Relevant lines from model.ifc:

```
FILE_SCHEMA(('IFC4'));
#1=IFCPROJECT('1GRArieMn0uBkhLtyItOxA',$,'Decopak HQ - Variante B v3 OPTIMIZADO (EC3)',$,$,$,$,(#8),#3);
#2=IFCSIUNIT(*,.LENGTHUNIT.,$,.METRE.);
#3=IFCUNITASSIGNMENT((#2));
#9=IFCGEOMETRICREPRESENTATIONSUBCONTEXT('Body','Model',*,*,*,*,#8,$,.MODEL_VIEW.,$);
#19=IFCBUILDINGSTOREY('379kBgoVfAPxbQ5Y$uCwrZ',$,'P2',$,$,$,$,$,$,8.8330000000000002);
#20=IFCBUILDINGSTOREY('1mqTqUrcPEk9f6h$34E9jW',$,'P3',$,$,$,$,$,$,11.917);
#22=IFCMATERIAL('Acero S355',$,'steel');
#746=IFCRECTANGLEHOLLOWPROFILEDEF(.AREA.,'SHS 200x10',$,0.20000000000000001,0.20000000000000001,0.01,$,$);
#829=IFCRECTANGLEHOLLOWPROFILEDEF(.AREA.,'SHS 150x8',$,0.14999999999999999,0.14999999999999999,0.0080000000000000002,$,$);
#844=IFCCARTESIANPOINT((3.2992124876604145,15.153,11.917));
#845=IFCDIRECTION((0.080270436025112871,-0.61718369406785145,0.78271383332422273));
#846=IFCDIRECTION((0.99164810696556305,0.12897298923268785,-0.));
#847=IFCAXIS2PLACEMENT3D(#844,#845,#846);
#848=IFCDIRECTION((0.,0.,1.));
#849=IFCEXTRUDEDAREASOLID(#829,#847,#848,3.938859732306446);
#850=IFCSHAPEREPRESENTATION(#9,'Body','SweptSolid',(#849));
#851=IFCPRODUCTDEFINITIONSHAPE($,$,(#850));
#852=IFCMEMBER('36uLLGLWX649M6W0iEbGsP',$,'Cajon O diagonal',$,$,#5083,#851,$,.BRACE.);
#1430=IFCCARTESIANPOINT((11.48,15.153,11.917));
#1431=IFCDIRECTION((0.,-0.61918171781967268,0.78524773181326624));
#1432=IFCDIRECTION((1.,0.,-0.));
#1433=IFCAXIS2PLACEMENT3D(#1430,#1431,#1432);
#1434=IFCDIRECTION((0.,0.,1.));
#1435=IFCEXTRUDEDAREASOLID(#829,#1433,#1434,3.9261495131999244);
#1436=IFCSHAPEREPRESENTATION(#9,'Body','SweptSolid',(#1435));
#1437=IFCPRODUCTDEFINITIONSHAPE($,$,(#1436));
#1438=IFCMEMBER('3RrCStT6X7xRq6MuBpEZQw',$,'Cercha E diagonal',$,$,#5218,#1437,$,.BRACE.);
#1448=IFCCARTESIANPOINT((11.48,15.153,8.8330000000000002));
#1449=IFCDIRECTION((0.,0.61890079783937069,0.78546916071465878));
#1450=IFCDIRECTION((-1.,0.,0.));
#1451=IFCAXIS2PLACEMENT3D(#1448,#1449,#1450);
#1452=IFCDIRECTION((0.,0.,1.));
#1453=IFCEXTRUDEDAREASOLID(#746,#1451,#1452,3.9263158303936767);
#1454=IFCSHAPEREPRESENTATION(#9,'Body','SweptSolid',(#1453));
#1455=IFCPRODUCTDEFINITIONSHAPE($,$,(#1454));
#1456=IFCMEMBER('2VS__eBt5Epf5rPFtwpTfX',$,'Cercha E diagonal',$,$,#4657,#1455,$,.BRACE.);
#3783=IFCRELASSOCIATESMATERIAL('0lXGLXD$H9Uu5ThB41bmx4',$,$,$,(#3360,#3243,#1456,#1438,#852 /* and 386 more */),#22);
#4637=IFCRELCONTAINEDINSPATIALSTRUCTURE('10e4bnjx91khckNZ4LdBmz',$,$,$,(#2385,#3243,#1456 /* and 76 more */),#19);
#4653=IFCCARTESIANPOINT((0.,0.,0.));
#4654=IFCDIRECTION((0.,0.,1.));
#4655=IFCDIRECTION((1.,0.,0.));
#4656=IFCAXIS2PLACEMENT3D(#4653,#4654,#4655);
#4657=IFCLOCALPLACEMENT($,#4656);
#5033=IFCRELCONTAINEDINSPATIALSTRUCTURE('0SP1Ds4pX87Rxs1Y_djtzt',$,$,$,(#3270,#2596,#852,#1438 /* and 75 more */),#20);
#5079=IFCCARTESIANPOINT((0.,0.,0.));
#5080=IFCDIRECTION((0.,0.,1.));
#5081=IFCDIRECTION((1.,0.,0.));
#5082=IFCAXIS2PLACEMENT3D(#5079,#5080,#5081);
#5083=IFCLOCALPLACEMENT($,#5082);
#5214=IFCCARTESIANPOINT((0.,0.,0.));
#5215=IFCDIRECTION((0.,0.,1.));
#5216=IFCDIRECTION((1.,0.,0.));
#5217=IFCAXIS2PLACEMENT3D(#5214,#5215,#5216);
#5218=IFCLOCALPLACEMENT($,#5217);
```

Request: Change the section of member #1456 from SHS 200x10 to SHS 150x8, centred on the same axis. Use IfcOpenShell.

```python
import ifcopenshell
import ifcopenshell.util.element
import ifcopenshell.util.representation

model = ifcopenshell.open("model.ifc")

member = model.by_id(1456)
source = next(p for p in model.by_type("IfcRectangleHollowProfileDef") if p.ProfileName == "SHS 150x8")

body = ifcopenshell.util.representation.get_representation(member, "Model", "Body")
solid = body.Items[0]
old_profile = solid.SweptArea

# Copy the section's sizes but keep this member's own profile position.
profile = ifcopenshell.util.element.copy(model, source)
profile.Position = old_profile.Position
solid.SweptArea = profile
if not model.get_total_inverses(old_profile):
    ifcopenshell.util.element.remove_deep2(model, old_profile)

print(solid.SweptArea)

model.write("model_updated.ifc")
```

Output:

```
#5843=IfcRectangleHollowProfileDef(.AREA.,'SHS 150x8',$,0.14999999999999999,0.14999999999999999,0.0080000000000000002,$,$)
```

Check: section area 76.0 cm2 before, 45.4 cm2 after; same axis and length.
